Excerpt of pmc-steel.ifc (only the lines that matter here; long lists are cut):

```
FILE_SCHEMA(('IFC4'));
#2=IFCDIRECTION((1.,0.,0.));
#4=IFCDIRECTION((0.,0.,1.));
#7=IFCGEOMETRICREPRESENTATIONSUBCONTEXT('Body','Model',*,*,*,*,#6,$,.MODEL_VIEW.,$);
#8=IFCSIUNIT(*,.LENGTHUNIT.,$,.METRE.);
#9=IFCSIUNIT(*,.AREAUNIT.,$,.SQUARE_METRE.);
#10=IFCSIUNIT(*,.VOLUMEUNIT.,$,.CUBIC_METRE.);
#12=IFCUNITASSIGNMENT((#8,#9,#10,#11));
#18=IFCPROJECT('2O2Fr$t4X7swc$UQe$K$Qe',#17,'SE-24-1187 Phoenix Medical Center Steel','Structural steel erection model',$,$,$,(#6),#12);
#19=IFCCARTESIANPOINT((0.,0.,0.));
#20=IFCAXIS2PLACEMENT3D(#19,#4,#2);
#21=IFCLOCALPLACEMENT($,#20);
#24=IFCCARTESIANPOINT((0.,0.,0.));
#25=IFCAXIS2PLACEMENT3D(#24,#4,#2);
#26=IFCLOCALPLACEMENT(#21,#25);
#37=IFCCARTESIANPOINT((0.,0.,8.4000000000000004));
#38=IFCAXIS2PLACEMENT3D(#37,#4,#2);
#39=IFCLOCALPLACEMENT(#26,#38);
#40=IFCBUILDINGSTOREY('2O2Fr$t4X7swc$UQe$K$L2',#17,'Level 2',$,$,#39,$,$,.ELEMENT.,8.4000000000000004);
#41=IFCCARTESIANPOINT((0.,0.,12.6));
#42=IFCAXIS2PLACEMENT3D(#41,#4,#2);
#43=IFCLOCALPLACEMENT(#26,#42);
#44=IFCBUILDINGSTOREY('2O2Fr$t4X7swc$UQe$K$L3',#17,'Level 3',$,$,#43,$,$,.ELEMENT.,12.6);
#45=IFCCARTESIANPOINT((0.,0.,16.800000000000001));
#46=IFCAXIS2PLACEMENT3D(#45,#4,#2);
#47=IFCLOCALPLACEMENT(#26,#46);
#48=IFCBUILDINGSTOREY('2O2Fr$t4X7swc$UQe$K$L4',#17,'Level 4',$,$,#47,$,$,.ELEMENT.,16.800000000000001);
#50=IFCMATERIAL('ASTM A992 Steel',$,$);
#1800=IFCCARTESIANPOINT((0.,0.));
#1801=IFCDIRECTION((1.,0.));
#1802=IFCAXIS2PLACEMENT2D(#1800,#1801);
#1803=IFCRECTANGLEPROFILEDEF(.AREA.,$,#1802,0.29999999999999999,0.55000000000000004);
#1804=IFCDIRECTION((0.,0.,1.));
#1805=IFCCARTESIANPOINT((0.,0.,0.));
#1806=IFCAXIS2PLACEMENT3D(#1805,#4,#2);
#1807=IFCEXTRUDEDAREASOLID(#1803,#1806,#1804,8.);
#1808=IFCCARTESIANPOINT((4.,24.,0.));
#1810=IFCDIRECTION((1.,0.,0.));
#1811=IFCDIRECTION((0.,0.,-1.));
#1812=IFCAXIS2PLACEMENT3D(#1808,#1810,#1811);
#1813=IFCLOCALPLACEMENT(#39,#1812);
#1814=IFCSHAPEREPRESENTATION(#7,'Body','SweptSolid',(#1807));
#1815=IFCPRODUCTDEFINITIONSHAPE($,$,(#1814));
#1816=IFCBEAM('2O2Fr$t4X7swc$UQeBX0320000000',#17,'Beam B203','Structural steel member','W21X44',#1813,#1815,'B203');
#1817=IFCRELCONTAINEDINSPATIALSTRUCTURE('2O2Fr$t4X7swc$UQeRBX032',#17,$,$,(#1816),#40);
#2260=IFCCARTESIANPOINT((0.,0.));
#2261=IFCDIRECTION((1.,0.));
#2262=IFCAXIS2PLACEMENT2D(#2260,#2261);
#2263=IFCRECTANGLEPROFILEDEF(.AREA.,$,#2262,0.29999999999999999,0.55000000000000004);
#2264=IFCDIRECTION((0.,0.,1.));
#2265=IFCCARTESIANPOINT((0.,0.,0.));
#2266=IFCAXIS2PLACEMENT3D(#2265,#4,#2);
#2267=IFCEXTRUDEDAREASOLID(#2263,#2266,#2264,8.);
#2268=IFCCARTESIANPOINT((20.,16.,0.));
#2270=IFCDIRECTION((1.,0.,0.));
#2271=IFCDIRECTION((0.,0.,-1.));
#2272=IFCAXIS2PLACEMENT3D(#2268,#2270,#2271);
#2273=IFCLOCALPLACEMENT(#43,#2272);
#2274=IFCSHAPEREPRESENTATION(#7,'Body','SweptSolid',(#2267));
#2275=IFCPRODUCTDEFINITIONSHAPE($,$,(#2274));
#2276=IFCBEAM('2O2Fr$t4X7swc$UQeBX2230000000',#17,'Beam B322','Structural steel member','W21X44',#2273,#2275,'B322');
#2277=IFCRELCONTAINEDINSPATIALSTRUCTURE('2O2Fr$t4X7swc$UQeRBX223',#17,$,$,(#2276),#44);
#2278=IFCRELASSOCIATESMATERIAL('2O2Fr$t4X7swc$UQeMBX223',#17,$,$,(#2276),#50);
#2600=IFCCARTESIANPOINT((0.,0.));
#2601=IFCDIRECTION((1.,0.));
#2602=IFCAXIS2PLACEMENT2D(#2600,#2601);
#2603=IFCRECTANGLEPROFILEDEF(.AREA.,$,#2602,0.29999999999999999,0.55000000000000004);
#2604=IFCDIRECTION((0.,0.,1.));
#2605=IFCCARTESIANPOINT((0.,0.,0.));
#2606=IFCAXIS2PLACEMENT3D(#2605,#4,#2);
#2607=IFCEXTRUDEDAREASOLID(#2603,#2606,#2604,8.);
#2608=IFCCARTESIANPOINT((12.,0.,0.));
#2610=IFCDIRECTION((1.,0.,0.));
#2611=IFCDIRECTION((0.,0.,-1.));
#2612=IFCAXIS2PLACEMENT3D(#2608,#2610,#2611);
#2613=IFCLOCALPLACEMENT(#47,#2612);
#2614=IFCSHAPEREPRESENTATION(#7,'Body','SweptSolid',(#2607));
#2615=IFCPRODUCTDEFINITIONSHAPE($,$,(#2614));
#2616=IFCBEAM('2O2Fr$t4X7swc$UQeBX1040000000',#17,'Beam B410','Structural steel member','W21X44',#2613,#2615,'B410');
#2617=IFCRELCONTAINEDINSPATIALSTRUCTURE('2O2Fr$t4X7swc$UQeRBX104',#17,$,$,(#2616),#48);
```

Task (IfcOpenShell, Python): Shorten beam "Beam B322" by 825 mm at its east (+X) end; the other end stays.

```python
import ifcopenshell
import ifcopenshell.util.representation
import ifcopenshell.util.unit

model = ifcopenshell.open("pmc-steel.ifc")
unit_scale = ifcopenshell.util.unit.calculate_unit_scale(model)

member = model.by_id(2276)
change = -0.825 / unit_scale

# The extrusion runs towards the end named, so only its depth changes.
body = ifcopenshell.util.representation.get_representation(member, "Model", "Body")
solid = body.Items[0]
old_length = solid.Depth
solid.Depth += change

print(f"length {old_length:g} -> {solid.Depth:g}")

model.write("pmc-steel_updated.ifc")
```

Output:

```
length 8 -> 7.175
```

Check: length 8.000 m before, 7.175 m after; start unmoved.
